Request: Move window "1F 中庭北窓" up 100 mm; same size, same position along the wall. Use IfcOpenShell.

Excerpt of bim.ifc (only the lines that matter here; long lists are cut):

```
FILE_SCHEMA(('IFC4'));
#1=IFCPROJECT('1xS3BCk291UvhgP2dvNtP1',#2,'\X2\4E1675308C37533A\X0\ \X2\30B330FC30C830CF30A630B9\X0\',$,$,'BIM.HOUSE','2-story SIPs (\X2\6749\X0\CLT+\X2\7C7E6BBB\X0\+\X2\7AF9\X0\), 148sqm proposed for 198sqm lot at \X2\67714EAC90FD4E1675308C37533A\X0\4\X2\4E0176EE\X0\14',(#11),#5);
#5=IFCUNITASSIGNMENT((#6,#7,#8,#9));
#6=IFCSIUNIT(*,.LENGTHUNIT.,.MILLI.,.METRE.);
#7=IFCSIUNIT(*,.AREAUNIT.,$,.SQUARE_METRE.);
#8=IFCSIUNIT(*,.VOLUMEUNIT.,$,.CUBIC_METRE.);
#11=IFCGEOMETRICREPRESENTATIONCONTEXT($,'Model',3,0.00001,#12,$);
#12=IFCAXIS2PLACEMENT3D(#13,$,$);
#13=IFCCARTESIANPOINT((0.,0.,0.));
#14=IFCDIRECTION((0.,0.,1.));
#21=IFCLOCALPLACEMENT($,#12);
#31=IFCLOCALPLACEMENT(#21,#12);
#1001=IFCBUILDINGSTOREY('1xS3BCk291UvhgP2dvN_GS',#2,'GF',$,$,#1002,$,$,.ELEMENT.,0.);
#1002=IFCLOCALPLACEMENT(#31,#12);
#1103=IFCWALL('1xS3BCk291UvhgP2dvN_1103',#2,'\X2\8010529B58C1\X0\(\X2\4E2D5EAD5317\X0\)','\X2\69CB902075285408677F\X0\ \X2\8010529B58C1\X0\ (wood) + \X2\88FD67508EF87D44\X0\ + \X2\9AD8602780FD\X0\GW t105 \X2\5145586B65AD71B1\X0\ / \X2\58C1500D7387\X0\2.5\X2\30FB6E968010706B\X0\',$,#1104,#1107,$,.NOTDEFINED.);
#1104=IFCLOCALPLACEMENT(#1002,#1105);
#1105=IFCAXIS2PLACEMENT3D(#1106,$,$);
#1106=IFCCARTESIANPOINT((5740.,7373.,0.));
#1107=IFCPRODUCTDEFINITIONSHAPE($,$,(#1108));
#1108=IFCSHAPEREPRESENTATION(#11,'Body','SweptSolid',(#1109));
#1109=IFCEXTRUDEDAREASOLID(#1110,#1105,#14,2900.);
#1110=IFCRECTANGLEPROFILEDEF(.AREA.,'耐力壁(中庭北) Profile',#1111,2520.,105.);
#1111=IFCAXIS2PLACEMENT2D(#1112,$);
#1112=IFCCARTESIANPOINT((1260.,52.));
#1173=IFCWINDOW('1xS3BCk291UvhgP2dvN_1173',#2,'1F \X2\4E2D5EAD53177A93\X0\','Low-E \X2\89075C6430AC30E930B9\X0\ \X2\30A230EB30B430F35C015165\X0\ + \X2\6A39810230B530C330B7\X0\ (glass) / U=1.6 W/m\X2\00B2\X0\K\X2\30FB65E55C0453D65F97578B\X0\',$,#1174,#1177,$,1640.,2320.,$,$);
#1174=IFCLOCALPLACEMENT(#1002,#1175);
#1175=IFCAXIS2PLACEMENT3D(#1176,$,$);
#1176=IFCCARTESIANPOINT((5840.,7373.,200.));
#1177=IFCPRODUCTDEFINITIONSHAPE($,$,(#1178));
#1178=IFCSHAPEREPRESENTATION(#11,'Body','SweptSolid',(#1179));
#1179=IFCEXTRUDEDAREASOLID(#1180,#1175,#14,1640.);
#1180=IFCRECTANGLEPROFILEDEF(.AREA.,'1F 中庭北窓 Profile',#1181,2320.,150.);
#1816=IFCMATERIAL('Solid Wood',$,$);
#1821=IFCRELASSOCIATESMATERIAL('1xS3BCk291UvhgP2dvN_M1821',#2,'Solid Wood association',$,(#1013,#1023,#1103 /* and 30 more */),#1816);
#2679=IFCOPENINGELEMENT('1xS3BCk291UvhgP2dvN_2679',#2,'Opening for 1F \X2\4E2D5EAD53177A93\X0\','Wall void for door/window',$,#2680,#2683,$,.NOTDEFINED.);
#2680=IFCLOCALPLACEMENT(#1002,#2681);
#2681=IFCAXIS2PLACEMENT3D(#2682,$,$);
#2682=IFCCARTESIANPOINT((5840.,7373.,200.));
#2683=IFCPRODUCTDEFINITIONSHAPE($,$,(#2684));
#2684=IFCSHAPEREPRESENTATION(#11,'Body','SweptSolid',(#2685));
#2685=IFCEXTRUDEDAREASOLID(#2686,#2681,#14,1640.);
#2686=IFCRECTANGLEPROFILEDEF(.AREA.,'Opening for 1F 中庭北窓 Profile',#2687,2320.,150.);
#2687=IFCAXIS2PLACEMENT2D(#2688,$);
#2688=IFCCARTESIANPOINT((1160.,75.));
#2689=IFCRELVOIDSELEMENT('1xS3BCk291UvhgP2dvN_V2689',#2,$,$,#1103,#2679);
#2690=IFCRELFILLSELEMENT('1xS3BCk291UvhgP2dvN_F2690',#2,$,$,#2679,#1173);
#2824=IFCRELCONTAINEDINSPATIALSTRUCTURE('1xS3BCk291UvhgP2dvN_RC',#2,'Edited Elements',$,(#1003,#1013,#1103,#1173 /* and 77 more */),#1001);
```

```python
import numpy as np
import ifcopenshell
import ifcopenshell.api.geometry
import ifcopenshell.util.placement
import ifcopenshell.util.unit

model = ifcopenshell.open("bim.ifc")
unit_scale = ifcopenshell.util.unit.calculate_unit_scale(model)

window = model.by_id(1173)
opening = window.FillsVoids[0].RelatingOpeningElement
dz = 0.1 / unit_scale

shift = np.array([0.0, 0.0, dz])
# The window is not placed relative to its opening, so move both.
for product in (opening, window):
    matrix = ifcopenshell.util.placement.get_local_placement(product.ObjectPlacement)
    matrix[:3, 3] += shift
    ifcopenshell.api.geometry.edit_object_placement(model, product=product, matrix=matrix, is_si=False)

print(f"moved by {dz * unit_scale:+.3f} m")

model.write("bim_updated.ifc")
```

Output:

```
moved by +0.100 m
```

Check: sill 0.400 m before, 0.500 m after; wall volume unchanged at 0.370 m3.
